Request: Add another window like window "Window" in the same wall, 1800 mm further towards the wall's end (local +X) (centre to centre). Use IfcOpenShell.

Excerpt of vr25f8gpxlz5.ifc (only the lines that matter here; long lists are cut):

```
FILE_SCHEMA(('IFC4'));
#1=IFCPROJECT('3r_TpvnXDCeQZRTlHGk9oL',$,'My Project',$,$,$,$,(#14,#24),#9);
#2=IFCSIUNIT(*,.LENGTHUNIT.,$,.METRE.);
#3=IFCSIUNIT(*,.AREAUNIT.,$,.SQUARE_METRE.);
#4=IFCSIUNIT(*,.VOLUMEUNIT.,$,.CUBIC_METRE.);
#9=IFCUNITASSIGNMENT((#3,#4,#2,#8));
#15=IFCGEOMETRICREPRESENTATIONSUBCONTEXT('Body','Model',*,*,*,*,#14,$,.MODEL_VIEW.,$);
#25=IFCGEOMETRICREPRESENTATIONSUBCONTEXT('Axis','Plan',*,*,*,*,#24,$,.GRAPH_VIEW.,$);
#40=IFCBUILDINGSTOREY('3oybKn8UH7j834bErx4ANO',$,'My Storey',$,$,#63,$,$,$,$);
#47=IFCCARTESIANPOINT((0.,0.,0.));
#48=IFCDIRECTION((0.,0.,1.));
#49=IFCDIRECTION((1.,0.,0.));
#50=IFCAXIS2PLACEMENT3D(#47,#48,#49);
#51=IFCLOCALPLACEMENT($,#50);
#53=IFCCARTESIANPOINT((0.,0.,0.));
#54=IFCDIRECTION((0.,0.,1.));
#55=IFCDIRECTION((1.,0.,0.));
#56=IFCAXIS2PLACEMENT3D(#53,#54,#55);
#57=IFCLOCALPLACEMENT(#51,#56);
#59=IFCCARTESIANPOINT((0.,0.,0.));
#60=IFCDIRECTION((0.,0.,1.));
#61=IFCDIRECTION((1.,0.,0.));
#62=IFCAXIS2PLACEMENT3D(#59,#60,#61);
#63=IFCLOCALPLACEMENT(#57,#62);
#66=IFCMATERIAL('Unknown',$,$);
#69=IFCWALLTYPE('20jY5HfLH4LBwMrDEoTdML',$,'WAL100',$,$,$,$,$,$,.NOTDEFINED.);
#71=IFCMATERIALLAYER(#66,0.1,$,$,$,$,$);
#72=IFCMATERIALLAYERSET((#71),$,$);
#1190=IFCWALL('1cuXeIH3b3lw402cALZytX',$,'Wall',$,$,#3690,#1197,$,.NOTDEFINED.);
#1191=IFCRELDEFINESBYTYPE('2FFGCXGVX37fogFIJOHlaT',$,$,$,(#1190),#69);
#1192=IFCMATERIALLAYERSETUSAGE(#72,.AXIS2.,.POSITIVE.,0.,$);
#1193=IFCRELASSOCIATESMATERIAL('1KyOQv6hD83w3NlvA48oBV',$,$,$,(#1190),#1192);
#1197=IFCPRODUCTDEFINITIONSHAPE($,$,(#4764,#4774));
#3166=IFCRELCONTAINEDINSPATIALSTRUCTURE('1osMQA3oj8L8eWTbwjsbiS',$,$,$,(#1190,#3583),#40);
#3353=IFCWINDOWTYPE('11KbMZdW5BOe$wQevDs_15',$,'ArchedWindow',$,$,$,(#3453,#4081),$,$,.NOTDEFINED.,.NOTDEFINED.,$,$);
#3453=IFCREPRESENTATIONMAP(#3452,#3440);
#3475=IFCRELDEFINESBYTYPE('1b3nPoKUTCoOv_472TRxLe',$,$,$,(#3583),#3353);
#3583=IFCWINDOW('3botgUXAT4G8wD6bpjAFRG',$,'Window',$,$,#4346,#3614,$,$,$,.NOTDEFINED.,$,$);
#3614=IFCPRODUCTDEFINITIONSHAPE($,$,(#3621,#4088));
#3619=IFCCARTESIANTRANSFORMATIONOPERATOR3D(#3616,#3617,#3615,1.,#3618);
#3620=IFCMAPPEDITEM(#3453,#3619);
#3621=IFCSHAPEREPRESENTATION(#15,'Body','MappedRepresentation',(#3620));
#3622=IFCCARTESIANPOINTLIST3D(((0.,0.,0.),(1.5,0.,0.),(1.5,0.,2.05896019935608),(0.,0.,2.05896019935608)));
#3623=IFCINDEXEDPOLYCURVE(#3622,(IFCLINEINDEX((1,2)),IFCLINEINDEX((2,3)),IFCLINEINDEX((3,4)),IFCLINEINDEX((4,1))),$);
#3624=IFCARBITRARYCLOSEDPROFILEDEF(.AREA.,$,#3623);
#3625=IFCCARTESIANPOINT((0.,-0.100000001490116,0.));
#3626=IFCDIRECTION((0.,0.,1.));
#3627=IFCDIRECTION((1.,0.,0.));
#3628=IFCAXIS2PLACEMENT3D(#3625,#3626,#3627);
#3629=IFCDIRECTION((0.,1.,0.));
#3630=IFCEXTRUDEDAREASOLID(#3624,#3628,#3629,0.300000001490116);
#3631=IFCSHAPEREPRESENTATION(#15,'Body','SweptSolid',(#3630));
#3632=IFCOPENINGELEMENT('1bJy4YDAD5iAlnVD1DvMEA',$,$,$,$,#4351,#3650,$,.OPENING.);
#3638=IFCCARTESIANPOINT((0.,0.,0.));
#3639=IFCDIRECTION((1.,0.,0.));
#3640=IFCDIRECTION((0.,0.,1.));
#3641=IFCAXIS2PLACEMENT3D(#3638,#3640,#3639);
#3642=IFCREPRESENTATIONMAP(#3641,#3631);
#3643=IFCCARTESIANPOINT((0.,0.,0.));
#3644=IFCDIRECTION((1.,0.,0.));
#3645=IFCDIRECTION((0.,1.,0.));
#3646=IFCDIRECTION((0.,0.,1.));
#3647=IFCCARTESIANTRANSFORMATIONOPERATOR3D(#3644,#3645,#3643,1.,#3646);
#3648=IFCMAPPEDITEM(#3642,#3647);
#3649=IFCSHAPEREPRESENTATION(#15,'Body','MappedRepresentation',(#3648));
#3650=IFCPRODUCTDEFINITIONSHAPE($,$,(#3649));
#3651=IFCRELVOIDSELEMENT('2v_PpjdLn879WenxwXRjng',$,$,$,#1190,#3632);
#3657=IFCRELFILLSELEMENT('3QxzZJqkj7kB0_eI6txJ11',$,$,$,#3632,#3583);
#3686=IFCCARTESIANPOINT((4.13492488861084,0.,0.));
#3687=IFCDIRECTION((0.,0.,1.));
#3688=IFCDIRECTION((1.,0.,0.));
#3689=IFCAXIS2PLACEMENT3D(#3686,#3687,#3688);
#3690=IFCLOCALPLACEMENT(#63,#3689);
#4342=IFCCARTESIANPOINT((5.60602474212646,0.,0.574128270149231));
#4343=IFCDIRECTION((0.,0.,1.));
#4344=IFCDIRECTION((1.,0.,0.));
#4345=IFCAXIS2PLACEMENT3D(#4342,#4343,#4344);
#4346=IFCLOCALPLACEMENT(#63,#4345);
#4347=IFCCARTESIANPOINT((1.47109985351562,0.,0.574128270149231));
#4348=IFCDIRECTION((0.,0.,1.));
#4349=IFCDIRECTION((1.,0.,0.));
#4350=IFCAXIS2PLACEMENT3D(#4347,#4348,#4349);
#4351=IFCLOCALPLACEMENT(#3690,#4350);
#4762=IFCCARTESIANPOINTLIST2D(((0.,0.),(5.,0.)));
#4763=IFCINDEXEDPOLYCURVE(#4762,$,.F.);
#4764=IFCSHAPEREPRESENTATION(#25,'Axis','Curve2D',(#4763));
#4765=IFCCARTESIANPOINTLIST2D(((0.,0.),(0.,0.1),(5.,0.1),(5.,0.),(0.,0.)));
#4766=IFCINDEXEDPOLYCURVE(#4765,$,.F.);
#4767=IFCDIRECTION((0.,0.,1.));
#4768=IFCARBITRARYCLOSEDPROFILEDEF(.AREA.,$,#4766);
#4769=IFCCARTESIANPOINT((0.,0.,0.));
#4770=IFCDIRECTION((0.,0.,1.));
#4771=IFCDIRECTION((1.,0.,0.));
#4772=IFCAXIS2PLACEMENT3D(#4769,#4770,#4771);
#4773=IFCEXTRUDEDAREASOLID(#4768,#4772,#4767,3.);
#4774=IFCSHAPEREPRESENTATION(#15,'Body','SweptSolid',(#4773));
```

```python
import ifcopenshell
import ifcopenshell.api.feature
import ifcopenshell.api.geometry
import ifcopenshell.api.root
import ifcopenshell.geom
import ifcopenshell.util.element
import ifcopenshell.util.placement
import ifcopenshell.util.shape

model = ifcopenshell.open("vr25f8gpxlz5.ifc")
settings = ifcopenshell.geom.settings()


def volume(element):
    """Net volume in cubic metres, openings subtracted."""
    shape = ifcopenshell.geom.create_shape(settings, element)
    return ifcopenshell.util.shape.get_volume(shape.geometry)


window = model.by_id(3583)
opening = window.FillsVoids[0].RelatingOpeningElement
wall = opening.VoidsElements[0].RelatingBuildingElement
before = volume(wall)
shift = ifcopenshell.util.placement.get_local_placement(wall.ObjectPlacement)[:3, 0] * 1.8

# copy_class copies the void relationship, type, container and properties, but no geometry.
new_opening = ifcopenshell.api.root.copy_class(model, product=opening)
new_opening.Representation = ifcopenshell.util.element.copy_deep(
    model, opening.Representation, exclude=["IfcGeometricRepresentationContext", "IfcRepresentationMap"]
)
new_window = ifcopenshell.api.root.copy_class(model, product=window)
new_window.Representation = ifcopenshell.util.element.copy_deep(
    model, window.Representation, exclude=["IfcGeometricRepresentationContext", "IfcRepresentationMap"]
)
ifcopenshell.api.feature.add_filling(model, opening=new_opening, element=new_window)

for old, new in ((opening, new_opening), (window, new_window)):
    matrix = ifcopenshell.util.placement.get_local_placement(old.ObjectPlacement)
    matrix[:3, 3] += shift
    ifcopenshell.api.geometry.edit_object_placement(model, product=new, matrix=matrix, is_si=False)

after = volume(wall)

print(f"wall volume {before:.3f} -> {after:.3f} m3")

model.write("vr25f8gpxlz5_edited.ifc")
```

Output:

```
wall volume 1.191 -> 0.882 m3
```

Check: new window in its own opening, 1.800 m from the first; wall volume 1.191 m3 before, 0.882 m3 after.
